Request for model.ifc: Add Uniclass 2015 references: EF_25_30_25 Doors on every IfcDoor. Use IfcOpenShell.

First a look at what the model holds.

```python
import ifcopenshell

model = ifcopenshell.open("model.ifc")
print(model.schema)
print("classifications:", [c.Name for c in model.by_type("IfcClassification")])
for ifc_class in ("IfcDoor", "IfcRoof", "IfcStair", "IfcWall", "IfcWindow"):
    print(ifc_class, len(model.by_type(ifc_class)))
```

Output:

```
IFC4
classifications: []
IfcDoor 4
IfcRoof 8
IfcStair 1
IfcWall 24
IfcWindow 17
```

```python
import ifcopenshell
import ifcopenshell.api.classification

model = ifcopenshell.open("model.ifc")

system = ifcopenshell.api.classification.add_classification(model, classification="Uniclass 2015")

codes = {
    "IfcDoor": ("EF_25_30_25", "Doors"),
}
for ifc_class, (code, name) in codes.items():
    products = model.by_type(ifc_class)
    ifcopenshell.api.classification.add_reference(
        model, products=products, classification=system, identification=code, name=name
    )
    print(code, len(products))

model.write("model_v2.ifc")
```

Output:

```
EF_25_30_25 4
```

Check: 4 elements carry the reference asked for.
